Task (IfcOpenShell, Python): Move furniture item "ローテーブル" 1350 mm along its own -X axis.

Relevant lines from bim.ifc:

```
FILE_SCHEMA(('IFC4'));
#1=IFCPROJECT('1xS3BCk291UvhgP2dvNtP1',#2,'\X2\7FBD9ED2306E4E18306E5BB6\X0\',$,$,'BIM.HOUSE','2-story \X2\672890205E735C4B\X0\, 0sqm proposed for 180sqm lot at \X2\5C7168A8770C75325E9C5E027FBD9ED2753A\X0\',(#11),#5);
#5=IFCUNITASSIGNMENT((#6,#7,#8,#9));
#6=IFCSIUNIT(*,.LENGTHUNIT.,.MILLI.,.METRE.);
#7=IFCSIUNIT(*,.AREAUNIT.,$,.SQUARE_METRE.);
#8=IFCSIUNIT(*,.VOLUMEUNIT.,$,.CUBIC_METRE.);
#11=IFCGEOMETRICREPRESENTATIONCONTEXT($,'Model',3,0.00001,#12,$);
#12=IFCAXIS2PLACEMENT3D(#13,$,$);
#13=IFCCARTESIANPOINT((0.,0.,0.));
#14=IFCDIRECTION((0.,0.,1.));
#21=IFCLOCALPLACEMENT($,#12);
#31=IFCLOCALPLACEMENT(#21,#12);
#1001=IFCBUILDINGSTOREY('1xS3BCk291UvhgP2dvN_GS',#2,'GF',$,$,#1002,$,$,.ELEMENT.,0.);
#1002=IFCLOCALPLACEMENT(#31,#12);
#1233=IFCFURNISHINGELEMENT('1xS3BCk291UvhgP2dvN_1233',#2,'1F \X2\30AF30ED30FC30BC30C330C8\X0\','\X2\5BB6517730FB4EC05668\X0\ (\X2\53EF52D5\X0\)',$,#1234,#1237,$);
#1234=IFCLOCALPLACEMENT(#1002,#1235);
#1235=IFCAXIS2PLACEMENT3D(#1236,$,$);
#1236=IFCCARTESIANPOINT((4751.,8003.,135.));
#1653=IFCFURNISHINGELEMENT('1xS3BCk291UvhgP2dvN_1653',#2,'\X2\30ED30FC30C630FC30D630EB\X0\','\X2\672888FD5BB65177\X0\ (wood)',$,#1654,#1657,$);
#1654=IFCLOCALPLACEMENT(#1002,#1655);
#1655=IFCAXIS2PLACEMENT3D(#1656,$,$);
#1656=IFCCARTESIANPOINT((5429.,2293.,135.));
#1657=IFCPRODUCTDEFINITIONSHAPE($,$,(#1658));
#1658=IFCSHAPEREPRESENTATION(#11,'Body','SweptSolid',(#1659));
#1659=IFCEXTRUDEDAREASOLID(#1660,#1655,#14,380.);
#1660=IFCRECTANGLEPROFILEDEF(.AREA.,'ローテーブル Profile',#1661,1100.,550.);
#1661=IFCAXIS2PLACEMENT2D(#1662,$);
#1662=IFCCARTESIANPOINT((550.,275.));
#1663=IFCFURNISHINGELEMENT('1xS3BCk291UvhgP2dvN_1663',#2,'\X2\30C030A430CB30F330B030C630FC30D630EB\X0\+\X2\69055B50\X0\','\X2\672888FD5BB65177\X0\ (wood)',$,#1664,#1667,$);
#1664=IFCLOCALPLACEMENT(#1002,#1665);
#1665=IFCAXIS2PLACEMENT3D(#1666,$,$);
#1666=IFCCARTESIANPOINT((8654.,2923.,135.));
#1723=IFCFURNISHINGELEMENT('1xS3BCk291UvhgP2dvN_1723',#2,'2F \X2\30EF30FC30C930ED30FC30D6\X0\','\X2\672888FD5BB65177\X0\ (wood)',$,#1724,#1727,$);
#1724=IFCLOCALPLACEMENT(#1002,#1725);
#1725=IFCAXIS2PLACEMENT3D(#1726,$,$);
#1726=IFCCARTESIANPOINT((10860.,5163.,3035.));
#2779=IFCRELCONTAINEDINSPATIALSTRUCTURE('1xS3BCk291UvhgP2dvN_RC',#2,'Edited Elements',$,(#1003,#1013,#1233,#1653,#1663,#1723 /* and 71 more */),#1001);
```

```python
import ifcopenshell
import ifcopenshell.api.geometry
import ifcopenshell.util.placement
import ifcopenshell.util.unit

model = ifcopenshell.open("bim.ifc")
unit_scale = ifcopenshell.util.unit.calculate_unit_scale(model)

item = model.by_guid("1xS3BCk291UvhgP2dvN_1653")
matrix = ifcopenshell.util.placement.get_local_placement(item.ObjectPlacement)
matrix[:3, 3] -= matrix[:3, 0] * 1.35 / unit_scale
ifcopenshell.api.geometry.edit_object_placement(model, product=item, matrix=matrix, is_si=False)

print(ifcopenshell.util.placement.get_local_placement(item.ObjectPlacement).round(3) + 0.0)

model.write("bim_v2.ifc")
```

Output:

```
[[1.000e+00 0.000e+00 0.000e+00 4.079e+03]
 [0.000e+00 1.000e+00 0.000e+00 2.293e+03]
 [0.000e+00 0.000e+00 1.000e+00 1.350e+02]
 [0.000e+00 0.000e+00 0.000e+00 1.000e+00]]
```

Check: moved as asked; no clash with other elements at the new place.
